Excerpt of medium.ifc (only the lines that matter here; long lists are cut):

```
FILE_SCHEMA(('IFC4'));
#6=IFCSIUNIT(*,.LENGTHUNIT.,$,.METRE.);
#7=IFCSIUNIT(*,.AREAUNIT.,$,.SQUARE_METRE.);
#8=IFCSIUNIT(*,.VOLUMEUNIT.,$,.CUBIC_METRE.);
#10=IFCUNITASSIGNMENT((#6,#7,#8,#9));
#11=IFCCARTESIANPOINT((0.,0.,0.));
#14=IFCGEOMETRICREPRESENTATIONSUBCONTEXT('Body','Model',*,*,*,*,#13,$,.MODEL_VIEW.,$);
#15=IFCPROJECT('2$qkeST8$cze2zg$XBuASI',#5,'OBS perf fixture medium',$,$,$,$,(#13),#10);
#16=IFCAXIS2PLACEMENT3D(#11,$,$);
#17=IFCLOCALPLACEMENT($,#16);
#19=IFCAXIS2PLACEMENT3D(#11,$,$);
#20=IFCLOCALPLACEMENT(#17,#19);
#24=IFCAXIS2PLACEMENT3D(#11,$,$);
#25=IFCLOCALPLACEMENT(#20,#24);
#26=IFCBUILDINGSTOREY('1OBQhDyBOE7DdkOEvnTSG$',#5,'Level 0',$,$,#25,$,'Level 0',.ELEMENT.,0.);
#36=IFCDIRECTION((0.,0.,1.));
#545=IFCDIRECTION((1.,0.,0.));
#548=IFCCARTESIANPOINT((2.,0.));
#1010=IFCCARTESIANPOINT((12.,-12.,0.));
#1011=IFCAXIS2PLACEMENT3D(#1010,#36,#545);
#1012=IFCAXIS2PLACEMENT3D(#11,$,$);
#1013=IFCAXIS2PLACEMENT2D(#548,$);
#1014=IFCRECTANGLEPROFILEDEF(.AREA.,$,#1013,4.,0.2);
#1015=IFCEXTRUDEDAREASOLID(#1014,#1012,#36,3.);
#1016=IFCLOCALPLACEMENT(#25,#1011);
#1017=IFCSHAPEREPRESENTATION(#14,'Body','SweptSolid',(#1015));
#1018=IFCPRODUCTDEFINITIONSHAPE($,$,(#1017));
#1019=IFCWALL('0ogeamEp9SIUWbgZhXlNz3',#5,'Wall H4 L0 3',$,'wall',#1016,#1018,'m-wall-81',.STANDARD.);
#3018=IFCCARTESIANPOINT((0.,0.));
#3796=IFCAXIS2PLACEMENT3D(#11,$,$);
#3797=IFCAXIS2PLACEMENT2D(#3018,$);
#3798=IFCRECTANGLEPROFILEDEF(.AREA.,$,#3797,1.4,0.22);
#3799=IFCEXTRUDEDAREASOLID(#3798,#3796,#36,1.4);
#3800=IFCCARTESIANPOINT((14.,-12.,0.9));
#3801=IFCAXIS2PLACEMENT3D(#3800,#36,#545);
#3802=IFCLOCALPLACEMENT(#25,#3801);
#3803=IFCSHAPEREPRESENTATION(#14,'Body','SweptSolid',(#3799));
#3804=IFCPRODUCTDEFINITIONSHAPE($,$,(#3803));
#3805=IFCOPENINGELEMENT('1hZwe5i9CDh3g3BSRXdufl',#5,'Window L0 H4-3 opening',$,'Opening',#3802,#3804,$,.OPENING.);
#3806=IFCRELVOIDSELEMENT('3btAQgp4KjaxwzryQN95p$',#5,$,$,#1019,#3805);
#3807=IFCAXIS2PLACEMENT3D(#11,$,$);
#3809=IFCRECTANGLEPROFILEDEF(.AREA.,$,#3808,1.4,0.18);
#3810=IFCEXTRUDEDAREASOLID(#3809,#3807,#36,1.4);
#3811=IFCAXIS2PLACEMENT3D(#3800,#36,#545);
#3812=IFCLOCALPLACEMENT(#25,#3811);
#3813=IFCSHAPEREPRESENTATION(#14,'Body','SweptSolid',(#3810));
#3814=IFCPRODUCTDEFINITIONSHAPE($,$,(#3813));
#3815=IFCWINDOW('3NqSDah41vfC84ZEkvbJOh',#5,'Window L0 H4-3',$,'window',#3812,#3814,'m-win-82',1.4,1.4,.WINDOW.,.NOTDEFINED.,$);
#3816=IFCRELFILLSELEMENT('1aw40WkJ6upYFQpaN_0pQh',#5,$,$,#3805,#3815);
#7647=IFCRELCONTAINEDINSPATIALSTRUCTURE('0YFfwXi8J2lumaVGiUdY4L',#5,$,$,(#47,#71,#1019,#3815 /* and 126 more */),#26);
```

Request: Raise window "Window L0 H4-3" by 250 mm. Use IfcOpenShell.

```python
import numpy as np
import ifcopenshell
import ifcopenshell.api.geometry
import ifcopenshell.util.placement
import ifcopenshell.util.unit

model = ifcopenshell.open("medium.ifc")
unit_scale = ifcopenshell.util.unit.calculate_unit_scale(model)

window = model.by_guid("3NqSDah41vfC84ZEkvbJOh")
opening = window.FillsVoids[0].RelatingOpeningElement
dz = 0.25 / unit_scale

shift = np.array([0.0, 0.0, dz])
# The window is not placed relative to its opening, so move both.
for product in (opening, window):
    matrix = ifcopenshell.util.placement.get_local_placement(product.ObjectPlacement)
    matrix[:3, 3] += shift
    ifcopenshell.api.geometry.edit_object_placement(model, product=product, matrix=matrix, is_si=False)

print(f"moved by {dz * unit_scale:+.3f} m")

model.write("medium_v2.ifc")
```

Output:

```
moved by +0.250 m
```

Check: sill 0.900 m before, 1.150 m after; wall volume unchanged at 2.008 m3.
